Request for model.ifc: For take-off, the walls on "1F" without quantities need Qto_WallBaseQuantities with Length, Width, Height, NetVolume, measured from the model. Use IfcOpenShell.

First a look at what the model holds.

```python
import ifcopenshell
import ifcopenshell.util.element
import ifcopenshell.util.unit

model = ifcopenshell.open("model.ifc")
print(model.schema)
for unit_type in ("LENGTHUNIT", "AREAUNIT", "VOLUMEUNIT"):
    print(unit_type, ifcopenshell.util.unit.calculate_unit_scale(model, unit_type))
storey = next(s for s in model.by_type("IfcBuildingStorey") if s.Name == "1F")
walls = [e for e in ifcopenshell.util.element.get_decomposition(storey) if e.is_a("IfcWall")]
for e in sorted(walls, key=lambda e: e.id()):
    print(e.id(), e.is_a(), e.Name, list(ifcopenshell.util.element.get_psets(e, qtos_only=True)), sep=" | ")
```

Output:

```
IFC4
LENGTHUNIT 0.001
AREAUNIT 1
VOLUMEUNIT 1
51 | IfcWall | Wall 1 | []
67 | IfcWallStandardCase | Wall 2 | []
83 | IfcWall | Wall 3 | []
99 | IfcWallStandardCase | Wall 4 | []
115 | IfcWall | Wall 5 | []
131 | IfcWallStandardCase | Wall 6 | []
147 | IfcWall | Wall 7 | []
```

```python
import ifcopenshell
import ifcopenshell.api.pset
import ifcopenshell.geom
import ifcopenshell.util.element
import ifcopenshell.util.shape
import ifcopenshell.util.unit

model = ifcopenshell.open("model.ifc")
unit_scale = ifcopenshell.util.unit.calculate_unit_scale(model)
volume_scale = ifcopenshell.util.unit.calculate_unit_scale(model, "VOLUMEUNIT")
settings = ifcopenshell.geom.settings()

storey = next(s for s in model.by_type("IfcBuildingStorey") if s.Name == "1F")
walls = [e for e in ifcopenshell.util.element.get_decomposition(storey) if e.is_a("IfcWall")]

for e in sorted(walls, key=lambda e: e.id()):
    if ifcopenshell.util.element.get_psets(e, qtos_only=True, should_inherit=False):
        continue
    # Geometry comes back in metres, in the element's own axes.
    shape = ifcopenshell.geom.create_shape(settings, e)
    values = {
        "Length": ifcopenshell.util.shape.get_x(shape.geometry) / unit_scale,
        "Width": ifcopenshell.util.shape.get_y(shape.geometry) / unit_scale,
        "Height": ifcopenshell.util.shape.get_z(shape.geometry) / unit_scale,
        "NetVolume": ifcopenshell.util.shape.get_volume(shape.geometry) / volume_scale,
    }
    qto = ifcopenshell.api.pset.add_qto(model, product=e, name="Qto_WallBaseQuantities")
    ifcopenshell.api.pset.edit_qto(model, qto=qto, properties=values)
    print(e.id(), {k: round(v, 3) for k, v in values.items()})

model.write("model_edited.ifc")
```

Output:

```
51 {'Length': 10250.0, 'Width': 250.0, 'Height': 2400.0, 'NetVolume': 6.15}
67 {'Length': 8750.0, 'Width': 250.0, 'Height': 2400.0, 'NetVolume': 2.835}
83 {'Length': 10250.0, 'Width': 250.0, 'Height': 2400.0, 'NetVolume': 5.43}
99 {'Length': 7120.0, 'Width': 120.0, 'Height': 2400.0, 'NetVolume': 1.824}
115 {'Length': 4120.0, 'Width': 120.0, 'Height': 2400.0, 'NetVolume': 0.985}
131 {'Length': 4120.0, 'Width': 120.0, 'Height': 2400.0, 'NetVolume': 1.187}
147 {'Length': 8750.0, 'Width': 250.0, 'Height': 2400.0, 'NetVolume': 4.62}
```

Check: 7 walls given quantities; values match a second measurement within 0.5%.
